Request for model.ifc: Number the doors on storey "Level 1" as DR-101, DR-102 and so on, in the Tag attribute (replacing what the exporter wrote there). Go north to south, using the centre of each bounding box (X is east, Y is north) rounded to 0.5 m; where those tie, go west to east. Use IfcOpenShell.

First a look at what the model holds.

```python
import ifcopenshell
import ifcopenshell.util.element
import ifcopenshell.util.placement

model = ifcopenshell.open("model.ifc")
print(model.schema)
storey = next(s for s in model.by_type("IfcBuildingStorey") if s.Name == "Level 1")
doors = [e for e in ifcopenshell.util.element.get_decomposition(storey) if e.is_a("IfcDoor")]
for e in sorted(doors, key=lambda e: e.id()):
    origin = ifcopenshell.util.placement.get_local_placement(e.ObjectPlacement)[:3, 3]
    print(e.id(), e.Tag, e.Name, origin.round(2) + 0.0, sep=" | ")
```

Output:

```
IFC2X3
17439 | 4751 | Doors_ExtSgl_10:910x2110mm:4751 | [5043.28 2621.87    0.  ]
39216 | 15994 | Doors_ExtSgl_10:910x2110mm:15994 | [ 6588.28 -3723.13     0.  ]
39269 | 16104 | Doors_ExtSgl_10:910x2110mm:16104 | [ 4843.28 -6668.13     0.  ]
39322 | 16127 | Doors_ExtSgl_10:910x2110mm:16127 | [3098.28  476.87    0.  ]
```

```python
import ifcopenshell
import ifcopenshell.geom
import ifcopenshell.util.element
import ifcopenshell.util.shape

model = ifcopenshell.open("model.ifc")
settings = ifcopenshell.geom.settings()
settings.set("use-world-coords", True)


def centre(element):
    shape = ifcopenshell.geom.create_shape(settings, element)
    return ifcopenshell.util.shape.get_bbox_centroid(shape.geometry)


storey = next(s for s in model.by_type("IfcBuildingStorey") if s.Name == "Level 1")
doors = [e for e in ifcopenshell.util.element.get_decomposition(storey) if e.is_a("IfcDoor")]

# Insertion points can sit at a corner or the storey origin, so sort by the geometry (in metres).
centres = {e: centre(e) for e in doors}
doors.sort(key=lambda e: (-round(centres[e][1] / 0.5), centres[e][0]))

for i, e in enumerate(doors, start=1):
    number = f"DR-1{i:02d}"
    e.Tag = number
    print(e.id(), number)

model.write("model_updated.ifc")
```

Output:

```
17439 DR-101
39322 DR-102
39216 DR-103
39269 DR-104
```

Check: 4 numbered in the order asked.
